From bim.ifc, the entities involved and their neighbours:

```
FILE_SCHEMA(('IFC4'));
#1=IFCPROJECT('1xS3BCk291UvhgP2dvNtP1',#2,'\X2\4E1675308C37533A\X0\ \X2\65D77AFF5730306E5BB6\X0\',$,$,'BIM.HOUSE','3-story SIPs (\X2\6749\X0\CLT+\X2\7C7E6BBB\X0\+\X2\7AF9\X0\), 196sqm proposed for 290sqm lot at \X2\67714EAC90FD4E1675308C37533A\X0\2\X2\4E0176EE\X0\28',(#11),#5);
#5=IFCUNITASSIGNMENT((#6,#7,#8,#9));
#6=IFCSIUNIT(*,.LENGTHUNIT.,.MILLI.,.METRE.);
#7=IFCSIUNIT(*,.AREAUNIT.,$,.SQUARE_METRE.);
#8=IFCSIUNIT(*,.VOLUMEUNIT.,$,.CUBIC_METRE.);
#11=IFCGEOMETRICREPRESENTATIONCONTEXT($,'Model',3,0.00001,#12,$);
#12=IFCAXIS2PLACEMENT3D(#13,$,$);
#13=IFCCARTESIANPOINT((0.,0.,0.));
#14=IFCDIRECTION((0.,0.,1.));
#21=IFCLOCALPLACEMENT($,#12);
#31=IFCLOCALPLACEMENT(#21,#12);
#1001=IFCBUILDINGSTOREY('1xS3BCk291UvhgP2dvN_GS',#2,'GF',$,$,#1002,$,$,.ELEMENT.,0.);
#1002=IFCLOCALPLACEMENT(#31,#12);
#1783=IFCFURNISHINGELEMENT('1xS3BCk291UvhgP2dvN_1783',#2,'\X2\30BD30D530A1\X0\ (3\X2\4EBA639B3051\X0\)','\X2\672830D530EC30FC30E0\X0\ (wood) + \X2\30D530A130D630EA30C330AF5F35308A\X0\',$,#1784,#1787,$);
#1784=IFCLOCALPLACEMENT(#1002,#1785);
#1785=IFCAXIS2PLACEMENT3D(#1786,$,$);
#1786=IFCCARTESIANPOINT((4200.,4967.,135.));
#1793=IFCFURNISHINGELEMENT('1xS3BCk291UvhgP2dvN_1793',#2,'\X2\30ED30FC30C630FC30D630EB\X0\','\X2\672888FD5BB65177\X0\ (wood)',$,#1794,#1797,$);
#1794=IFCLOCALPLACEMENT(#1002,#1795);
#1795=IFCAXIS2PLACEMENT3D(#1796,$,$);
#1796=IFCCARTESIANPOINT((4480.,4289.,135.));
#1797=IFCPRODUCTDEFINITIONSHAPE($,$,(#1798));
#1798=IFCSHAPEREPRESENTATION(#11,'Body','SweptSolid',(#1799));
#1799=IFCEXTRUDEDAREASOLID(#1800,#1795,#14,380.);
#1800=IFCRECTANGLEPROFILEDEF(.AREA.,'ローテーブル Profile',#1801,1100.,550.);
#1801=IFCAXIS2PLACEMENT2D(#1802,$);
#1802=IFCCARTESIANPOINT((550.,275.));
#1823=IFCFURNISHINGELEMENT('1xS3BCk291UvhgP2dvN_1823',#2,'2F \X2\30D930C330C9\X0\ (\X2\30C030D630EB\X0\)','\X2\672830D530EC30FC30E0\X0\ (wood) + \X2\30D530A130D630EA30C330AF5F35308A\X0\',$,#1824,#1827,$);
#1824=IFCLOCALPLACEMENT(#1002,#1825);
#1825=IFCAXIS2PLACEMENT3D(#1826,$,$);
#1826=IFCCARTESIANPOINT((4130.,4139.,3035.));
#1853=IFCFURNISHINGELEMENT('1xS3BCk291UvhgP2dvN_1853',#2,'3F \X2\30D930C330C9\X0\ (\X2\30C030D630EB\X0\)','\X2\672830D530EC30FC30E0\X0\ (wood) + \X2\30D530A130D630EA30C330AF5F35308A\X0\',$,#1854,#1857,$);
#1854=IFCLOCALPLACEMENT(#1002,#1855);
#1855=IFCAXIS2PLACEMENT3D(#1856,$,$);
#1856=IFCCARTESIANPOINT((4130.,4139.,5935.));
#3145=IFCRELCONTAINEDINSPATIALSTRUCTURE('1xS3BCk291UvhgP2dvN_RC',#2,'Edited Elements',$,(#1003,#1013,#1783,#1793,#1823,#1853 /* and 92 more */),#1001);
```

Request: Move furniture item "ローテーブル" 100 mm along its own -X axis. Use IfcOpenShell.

```python
import ifcopenshell
import ifcopenshell.api.geometry
import ifcopenshell.util.placement
import ifcopenshell.util.unit

model = ifcopenshell.open("bim.ifc")
unit_scale = ifcopenshell.util.unit.calculate_unit_scale(model)

item = model.by_id(1793)
matrix = ifcopenshell.util.placement.get_local_placement(item.ObjectPlacement)
matrix[:3, 3] -= matrix[:3, 0] * 0.1 / unit_scale
ifcopenshell.api.geometry.edit_object_placement(model, product=item, matrix=matrix, is_si=False)

print(ifcopenshell.util.placement.get_local_placement(item.ObjectPlacement).round(3) + 0.0)

model.write("bim_edited.ifc")
```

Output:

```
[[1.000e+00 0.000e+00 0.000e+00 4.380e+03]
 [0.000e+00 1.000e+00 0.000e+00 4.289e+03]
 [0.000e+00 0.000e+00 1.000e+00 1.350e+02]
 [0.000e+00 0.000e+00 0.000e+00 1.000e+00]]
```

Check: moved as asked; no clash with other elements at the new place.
